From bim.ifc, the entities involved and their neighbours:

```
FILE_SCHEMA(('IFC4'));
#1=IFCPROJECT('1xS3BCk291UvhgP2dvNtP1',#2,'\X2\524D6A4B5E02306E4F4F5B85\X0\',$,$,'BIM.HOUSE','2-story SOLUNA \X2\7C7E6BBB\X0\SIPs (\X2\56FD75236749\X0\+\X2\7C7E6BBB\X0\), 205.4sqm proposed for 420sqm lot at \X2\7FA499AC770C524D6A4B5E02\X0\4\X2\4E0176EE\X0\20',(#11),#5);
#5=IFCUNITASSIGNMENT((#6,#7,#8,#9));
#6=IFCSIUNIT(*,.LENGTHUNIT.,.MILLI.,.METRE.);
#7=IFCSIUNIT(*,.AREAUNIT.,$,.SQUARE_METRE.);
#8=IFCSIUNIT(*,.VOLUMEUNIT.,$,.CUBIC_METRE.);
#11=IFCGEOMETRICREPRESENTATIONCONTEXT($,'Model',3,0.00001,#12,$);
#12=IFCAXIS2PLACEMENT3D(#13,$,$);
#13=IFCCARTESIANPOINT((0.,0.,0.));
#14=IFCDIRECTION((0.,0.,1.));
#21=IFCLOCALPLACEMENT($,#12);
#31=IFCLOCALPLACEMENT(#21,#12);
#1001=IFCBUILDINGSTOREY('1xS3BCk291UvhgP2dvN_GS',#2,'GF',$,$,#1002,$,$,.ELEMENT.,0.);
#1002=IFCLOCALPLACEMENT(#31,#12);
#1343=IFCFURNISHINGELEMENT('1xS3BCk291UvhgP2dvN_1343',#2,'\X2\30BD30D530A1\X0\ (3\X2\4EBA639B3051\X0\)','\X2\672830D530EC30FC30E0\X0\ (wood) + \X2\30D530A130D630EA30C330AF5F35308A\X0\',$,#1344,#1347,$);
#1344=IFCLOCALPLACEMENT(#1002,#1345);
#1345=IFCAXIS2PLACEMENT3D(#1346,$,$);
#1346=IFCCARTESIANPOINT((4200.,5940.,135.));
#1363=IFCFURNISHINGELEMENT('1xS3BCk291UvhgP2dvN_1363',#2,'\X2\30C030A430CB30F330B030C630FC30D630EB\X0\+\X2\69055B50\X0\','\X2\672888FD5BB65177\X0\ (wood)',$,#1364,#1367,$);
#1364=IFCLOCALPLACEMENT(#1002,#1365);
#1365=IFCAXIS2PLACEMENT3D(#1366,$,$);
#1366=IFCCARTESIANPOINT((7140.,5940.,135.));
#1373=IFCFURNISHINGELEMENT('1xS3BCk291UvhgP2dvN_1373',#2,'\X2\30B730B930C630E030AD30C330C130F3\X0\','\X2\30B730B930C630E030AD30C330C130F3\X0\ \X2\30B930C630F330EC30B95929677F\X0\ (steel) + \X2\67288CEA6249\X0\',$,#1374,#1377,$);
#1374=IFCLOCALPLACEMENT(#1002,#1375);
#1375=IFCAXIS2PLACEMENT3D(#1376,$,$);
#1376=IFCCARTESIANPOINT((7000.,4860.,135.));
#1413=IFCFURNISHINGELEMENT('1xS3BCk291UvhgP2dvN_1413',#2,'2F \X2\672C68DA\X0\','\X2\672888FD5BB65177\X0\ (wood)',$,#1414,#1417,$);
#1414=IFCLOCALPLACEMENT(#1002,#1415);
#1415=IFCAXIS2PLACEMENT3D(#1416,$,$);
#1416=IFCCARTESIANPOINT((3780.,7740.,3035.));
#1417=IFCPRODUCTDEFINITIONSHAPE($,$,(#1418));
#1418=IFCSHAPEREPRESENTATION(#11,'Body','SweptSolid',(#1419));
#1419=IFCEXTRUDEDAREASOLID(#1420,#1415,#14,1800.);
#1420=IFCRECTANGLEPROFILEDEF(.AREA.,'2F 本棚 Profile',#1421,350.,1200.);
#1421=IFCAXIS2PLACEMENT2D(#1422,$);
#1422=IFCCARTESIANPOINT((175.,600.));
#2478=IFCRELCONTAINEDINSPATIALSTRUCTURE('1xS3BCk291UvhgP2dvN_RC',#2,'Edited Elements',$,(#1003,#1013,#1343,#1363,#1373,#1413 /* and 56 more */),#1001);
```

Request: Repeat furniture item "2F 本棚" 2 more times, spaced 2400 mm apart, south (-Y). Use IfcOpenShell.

```python
import numpy as np
import ifcopenshell
import ifcopenshell.api.geometry
import ifcopenshell.api.root
import ifcopenshell.util.element
import ifcopenshell.util.placement
import ifcopenshell.util.unit

model = ifcopenshell.open("bim.ifc")
unit_scale = ifcopenshell.util.unit.calculate_unit_scale(model)


def reuse_history(source, copy):
    """copy_class also copies each property set's owner history, people and application; keep the originals."""
    for rel in copy.IsDefinedBy:
        if rel.is_a("IfcRelDefinesByProperties") and (history := rel.RelatingPropertyDefinition.OwnerHistory):
            rel.RelatingPropertyDefinition.OwnerHistory = source.OwnerHistory
            ifcopenshell.util.element.remove_deep2(model, history)


source = model.by_guid("1xS3BCk291UvhgP2dvN_1413")
base = ifcopenshell.util.placement.get_local_placement(source.ObjectPlacement)
step = np.array([0.0, -1.0, 0.0]) * 2.4 / unit_scale

for i in range(1, 3):
    copy = ifcopenshell.api.root.copy_class(model, product=source)
    copy.Representation = ifcopenshell.util.element.copy_deep(
        model, source.Representation, exclude=["IfcGeometricRepresentationContext", "IfcRepresentationMap"]
    )
    reuse_history(source, copy)
    matrix = base.copy()
    matrix[:3, 3] += i * step
    print("added at", matrix[:3, 3].round(3) + 0.0)
    ifcopenshell.api.geometry.edit_object_placement(model, product=copy, matrix=matrix, is_si=False)

model.write("bim_rev.ifc")
```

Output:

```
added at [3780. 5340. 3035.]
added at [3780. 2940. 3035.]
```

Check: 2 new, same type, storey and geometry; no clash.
